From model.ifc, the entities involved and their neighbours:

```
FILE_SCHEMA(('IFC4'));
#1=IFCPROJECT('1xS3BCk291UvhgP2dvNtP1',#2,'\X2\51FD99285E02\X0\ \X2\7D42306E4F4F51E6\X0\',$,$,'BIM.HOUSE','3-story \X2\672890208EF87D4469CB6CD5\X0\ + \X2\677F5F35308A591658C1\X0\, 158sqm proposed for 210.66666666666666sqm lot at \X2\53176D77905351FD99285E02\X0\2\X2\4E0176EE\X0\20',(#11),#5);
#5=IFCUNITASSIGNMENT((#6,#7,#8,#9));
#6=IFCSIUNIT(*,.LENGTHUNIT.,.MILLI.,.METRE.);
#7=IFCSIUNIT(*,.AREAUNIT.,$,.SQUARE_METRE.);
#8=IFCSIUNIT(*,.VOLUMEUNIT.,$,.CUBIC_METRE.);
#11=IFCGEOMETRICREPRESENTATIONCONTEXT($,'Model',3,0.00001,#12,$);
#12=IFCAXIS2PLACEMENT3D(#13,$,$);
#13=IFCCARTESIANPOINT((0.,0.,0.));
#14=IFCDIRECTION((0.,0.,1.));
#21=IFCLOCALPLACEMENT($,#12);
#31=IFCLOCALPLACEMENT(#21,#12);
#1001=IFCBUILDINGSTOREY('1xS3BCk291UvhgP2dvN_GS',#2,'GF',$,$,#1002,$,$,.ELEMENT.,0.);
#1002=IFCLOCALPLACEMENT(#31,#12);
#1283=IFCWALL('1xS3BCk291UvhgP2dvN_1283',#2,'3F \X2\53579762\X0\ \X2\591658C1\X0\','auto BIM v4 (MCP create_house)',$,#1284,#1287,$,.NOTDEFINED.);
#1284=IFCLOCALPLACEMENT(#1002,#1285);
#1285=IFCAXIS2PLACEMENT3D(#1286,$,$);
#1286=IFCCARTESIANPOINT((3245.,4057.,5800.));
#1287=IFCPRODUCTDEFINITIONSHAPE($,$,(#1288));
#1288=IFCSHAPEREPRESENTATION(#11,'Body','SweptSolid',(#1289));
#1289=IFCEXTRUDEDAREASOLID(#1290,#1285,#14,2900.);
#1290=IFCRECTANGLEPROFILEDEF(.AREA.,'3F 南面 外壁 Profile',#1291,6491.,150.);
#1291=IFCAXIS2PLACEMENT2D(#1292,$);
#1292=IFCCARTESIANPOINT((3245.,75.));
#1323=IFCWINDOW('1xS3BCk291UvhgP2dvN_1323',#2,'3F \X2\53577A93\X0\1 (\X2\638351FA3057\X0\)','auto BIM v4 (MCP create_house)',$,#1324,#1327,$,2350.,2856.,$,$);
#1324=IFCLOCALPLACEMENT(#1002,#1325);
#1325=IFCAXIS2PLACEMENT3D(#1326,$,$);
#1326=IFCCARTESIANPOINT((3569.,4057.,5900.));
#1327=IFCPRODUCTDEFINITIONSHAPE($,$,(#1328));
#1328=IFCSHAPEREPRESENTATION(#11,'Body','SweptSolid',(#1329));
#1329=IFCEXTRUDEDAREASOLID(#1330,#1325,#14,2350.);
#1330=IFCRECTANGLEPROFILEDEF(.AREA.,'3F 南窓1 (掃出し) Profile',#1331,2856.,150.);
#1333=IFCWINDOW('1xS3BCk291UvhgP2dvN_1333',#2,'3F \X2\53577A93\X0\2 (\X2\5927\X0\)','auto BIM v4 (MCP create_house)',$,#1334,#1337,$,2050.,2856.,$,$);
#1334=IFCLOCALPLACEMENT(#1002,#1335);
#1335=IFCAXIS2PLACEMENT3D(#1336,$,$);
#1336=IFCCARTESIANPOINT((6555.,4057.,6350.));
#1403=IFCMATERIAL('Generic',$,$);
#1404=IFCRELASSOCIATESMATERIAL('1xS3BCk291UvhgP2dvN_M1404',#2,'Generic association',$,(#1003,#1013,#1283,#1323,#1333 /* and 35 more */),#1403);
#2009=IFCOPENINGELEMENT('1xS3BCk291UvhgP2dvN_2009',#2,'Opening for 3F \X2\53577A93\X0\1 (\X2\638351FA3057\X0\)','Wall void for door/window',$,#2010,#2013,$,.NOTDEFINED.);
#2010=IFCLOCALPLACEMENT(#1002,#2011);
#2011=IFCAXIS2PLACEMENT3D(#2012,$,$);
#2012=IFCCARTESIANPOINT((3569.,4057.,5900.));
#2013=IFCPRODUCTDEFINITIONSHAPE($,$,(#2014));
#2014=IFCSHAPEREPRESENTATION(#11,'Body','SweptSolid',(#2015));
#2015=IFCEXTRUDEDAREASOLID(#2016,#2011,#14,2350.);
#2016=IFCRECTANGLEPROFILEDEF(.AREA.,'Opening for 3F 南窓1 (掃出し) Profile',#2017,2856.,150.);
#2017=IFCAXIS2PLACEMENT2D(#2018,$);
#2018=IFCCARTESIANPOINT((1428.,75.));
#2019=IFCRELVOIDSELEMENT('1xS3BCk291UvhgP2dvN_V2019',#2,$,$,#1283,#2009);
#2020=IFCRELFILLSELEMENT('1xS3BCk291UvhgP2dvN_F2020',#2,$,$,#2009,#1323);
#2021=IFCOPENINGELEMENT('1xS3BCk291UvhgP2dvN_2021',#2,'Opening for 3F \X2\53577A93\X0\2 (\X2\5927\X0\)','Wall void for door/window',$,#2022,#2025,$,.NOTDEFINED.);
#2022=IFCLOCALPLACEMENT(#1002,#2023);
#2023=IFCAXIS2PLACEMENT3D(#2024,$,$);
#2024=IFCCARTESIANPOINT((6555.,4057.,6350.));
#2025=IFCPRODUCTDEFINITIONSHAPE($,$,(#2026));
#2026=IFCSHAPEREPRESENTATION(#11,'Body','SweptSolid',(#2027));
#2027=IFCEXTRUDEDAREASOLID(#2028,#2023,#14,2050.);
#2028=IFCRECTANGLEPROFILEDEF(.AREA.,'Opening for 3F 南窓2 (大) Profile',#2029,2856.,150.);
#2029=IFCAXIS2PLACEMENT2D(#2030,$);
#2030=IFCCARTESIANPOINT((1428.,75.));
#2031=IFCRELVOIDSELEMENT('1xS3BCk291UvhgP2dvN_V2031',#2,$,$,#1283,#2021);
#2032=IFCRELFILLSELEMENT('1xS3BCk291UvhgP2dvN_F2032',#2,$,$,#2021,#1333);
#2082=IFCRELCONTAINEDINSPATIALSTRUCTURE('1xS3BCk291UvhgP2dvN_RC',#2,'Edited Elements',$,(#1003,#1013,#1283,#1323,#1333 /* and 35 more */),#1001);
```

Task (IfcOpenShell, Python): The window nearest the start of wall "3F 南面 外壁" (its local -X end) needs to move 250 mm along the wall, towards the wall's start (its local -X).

```python
import ifcopenshell
import ifcopenshell.api.geometry
import ifcopenshell.util.placement

model = ifcopenshell.open("model.ifc")

window = model.by_id(1323)
opening = window.FillsVoids[0].RelatingOpeningElement
wall = opening.VoidsElements[0].RelatingBuildingElement

wall_matrix = ifcopenshell.util.placement.get_local_placement(wall.ObjectPlacement)
shift = wall_matrix[:3, 0] * -250.0
before = ifcopenshell.util.placement.get_local_placement(window.ObjectPlacement)[:3, 3].copy()

# The window is not placed relative to its opening, so move both.
for product in (opening, window):
    matrix = ifcopenshell.util.placement.get_local_placement(product.ObjectPlacement)
    matrix[:3, 3] += shift
    ifcopenshell.api.geometry.edit_object_placement(model, product=product, matrix=matrix, is_si=False)

after = ifcopenshell.util.placement.get_local_placement(window.ObjectPlacement)[:3, 3]
print("window moved by", (after - before).round(3) + 0.0)

model.write("model-out.ifc")
```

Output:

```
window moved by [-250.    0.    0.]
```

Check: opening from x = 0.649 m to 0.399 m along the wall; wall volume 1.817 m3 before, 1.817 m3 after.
